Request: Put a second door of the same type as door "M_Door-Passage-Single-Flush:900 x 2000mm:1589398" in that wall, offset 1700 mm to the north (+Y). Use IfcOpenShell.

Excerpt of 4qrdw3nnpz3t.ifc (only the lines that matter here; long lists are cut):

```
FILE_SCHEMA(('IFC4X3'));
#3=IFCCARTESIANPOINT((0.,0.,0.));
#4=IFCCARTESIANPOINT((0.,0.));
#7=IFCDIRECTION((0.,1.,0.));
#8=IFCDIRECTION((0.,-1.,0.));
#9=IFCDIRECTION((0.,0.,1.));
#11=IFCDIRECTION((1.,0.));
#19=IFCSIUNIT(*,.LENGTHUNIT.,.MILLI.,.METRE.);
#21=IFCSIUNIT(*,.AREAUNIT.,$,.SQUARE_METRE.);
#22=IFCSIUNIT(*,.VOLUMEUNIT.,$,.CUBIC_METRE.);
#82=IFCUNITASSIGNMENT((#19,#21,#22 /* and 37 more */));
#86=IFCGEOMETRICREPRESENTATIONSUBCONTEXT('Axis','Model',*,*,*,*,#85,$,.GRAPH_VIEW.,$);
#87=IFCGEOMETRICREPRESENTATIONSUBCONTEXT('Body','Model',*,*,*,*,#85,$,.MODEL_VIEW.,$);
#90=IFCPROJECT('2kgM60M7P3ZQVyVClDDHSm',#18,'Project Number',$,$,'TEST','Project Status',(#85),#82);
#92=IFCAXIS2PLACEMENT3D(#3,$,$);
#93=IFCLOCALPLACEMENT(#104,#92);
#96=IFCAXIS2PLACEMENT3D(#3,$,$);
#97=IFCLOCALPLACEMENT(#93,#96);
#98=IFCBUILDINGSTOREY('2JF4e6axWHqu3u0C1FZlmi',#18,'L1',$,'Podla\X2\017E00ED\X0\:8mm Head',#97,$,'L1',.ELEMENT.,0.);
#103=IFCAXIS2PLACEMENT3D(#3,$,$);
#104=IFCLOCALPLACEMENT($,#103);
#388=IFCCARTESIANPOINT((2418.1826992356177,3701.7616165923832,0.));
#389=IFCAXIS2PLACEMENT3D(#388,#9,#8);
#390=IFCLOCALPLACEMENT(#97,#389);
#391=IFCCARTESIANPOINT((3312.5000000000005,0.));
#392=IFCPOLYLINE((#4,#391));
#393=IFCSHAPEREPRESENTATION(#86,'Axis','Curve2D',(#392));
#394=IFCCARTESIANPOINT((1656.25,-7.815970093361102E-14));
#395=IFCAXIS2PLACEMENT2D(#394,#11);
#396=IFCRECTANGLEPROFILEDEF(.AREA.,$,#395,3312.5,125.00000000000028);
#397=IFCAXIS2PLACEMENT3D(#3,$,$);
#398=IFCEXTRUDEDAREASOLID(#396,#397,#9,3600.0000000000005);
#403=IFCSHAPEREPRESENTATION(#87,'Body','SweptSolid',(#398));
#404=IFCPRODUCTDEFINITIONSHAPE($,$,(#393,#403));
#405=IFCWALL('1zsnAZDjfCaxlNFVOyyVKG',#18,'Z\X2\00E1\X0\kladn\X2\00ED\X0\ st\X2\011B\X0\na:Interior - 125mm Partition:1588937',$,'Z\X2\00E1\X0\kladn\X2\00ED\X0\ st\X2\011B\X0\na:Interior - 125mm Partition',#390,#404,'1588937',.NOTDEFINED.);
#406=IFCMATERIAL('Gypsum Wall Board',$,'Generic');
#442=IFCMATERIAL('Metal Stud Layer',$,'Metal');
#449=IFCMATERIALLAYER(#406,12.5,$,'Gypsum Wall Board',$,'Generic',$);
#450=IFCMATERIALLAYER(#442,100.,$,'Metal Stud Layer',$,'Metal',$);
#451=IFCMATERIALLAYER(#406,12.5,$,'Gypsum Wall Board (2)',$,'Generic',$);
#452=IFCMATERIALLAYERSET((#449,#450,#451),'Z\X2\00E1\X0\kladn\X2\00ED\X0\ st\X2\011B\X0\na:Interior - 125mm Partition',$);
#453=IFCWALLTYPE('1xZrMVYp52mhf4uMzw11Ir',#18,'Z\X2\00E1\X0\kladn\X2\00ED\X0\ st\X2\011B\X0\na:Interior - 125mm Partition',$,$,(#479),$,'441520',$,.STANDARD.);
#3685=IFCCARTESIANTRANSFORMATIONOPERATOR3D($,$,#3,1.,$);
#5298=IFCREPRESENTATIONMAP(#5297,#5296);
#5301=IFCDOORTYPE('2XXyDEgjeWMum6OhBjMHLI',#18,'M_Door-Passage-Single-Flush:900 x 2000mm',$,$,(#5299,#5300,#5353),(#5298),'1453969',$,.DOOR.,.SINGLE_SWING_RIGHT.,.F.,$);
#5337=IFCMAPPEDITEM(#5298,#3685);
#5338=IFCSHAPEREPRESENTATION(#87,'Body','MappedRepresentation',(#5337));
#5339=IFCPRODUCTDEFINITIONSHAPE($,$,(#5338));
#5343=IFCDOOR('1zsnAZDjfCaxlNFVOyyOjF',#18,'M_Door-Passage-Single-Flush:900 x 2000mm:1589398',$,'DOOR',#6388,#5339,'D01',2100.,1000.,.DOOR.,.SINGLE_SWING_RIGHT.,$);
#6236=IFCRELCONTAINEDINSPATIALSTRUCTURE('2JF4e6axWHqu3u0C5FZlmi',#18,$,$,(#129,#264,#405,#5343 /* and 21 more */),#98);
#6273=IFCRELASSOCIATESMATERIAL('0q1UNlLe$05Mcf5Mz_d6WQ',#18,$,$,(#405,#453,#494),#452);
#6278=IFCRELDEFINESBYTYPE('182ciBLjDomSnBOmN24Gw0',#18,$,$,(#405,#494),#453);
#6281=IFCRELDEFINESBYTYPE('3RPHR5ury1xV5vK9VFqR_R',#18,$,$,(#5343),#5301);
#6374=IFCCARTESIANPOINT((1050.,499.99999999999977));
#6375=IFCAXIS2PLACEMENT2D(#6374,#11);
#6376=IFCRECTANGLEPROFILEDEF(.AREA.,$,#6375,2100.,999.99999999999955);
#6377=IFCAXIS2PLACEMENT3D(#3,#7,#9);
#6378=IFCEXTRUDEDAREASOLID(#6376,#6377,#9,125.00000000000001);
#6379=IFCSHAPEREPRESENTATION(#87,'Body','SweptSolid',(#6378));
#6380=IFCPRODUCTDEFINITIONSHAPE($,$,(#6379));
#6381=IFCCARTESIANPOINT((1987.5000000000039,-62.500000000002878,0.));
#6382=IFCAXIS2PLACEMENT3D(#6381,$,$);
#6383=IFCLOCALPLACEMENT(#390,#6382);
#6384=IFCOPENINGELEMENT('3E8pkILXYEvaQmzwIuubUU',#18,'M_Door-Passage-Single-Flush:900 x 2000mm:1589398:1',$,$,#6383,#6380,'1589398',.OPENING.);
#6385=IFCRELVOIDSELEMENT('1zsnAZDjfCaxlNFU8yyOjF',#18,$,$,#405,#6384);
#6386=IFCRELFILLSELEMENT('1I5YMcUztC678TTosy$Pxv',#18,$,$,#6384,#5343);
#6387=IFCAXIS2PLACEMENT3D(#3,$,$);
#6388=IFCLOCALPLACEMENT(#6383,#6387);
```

```python
import ifcopenshell
import ifcopenshell.api.feature
import ifcopenshell.api.geometry
import ifcopenshell.api.root
import ifcopenshell.geom
import ifcopenshell.util.element
import ifcopenshell.util.placement
import ifcopenshell.util.shape
import ifcopenshell.util.unit

model = ifcopenshell.open("4qrdw3nnpz3t.ifc")
unit_scale = ifcopenshell.util.unit.calculate_unit_scale(model)
settings = ifcopenshell.geom.settings()


def volume(element):
    """Net volume in cubic metres, openings subtracted."""
    shape = ifcopenshell.geom.create_shape(settings, element)
    return ifcopenshell.util.shape.get_volume(shape.geometry)


def reuse_history(source, copy):
    """copy_class also copies each property set's owner history, people and application; keep the originals."""
    for rel in copy.IsDefinedBy:
        if rel.is_a("IfcRelDefinesByProperties") and (history := rel.RelatingPropertyDefinition.OwnerHistory):
            rel.RelatingPropertyDefinition.OwnerHistory = source.OwnerHistory
            ifcopenshell.util.element.remove_deep2(model, history)


door = model.by_id(5343)
opening = door.FillsVoids[0].RelatingOpeningElement
wall = opening.VoidsElements[0].RelatingBuildingElement
before = volume(wall)
shift = ifcopenshell.util.placement.get_local_placement(wall.ObjectPlacement)[:3, 0] * -1.7 / unit_scale

# copy_class copies the void relationship, type, container and properties, but no geometry.
new_opening = ifcopenshell.api.root.copy_class(model, product=opening)
new_opening.Representation = ifcopenshell.util.element.copy_deep(
    model, opening.Representation, exclude=["IfcGeometricRepresentationContext", "IfcRepresentationMap"]
)
new_opening.Name = "M_Door-Passage-Single-Flush:900 x 2000mm"
new_opening.Tag = None
new_door = ifcopenshell.api.root.copy_class(model, product=door)
new_door.Representation = ifcopenshell.util.element.copy_deep(
    model, door.Representation, exclude=["IfcGeometricRepresentationContext", "IfcRepresentationMap"]
)
new_door.Name = "M_Door-Passage-Single-Flush:900 x 2000mm"
new_door.Tag = None
reuse_history(door, new_door)
ifcopenshell.api.feature.add_filling(model, opening=new_opening, element=new_door)

for old, new in ((opening, new_opening), (door, new_door)):
    matrix = ifcopenshell.util.placement.get_local_placement(old.ObjectPlacement)
    matrix[:3, 3] += shift
    ifcopenshell.api.geometry.edit_object_placement(model, product=new, matrix=matrix, is_si=False)

after = volume(wall)

print(f"wall volume {before:.3f} -> {after:.3f} m3")

model.write("4qrdw3nnpz3t_updated.ifc")
```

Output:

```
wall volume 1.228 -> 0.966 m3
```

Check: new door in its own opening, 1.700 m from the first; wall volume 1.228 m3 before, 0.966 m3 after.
